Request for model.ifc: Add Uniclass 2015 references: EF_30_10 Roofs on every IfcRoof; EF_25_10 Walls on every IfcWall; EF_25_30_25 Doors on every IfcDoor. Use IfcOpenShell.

First a look at what the model holds.

```python
import ifcopenshell

model = ifcopenshell.open("model.ifc")
print(model.schema)
print("classifications:", [c.Name for c in model.by_type("IfcClassification")])
for ifc_class in ("IfcDoor", "IfcRoof", "IfcStair", "IfcWall", "IfcWindow"):
    print(ifc_class, len(model.by_type(ifc_class)))
```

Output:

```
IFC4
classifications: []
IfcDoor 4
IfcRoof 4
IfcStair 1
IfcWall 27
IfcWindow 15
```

```python
import ifcopenshell
import ifcopenshell.api.classification

model = ifcopenshell.open("model.ifc")

system = ifcopenshell.api.classification.add_classification(model, classification="Uniclass 2015")

codes = {
    "IfcRoof": ("EF_30_10", "Roofs"),
    "IfcWall": ("EF_25_10", "Walls"),
    "IfcDoor": ("EF_25_30_25", "Doors"),
}
for ifc_class, (code, name) in codes.items():
    products = model.by_type(ifc_class)
    ifcopenshell.api.classification.add_reference(
        model, products=products, classification=system, identification=code, name=name
    )
    print(code, len(products))

model.write("model_edited.ifc")
```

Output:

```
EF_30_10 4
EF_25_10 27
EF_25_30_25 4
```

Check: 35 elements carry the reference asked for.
